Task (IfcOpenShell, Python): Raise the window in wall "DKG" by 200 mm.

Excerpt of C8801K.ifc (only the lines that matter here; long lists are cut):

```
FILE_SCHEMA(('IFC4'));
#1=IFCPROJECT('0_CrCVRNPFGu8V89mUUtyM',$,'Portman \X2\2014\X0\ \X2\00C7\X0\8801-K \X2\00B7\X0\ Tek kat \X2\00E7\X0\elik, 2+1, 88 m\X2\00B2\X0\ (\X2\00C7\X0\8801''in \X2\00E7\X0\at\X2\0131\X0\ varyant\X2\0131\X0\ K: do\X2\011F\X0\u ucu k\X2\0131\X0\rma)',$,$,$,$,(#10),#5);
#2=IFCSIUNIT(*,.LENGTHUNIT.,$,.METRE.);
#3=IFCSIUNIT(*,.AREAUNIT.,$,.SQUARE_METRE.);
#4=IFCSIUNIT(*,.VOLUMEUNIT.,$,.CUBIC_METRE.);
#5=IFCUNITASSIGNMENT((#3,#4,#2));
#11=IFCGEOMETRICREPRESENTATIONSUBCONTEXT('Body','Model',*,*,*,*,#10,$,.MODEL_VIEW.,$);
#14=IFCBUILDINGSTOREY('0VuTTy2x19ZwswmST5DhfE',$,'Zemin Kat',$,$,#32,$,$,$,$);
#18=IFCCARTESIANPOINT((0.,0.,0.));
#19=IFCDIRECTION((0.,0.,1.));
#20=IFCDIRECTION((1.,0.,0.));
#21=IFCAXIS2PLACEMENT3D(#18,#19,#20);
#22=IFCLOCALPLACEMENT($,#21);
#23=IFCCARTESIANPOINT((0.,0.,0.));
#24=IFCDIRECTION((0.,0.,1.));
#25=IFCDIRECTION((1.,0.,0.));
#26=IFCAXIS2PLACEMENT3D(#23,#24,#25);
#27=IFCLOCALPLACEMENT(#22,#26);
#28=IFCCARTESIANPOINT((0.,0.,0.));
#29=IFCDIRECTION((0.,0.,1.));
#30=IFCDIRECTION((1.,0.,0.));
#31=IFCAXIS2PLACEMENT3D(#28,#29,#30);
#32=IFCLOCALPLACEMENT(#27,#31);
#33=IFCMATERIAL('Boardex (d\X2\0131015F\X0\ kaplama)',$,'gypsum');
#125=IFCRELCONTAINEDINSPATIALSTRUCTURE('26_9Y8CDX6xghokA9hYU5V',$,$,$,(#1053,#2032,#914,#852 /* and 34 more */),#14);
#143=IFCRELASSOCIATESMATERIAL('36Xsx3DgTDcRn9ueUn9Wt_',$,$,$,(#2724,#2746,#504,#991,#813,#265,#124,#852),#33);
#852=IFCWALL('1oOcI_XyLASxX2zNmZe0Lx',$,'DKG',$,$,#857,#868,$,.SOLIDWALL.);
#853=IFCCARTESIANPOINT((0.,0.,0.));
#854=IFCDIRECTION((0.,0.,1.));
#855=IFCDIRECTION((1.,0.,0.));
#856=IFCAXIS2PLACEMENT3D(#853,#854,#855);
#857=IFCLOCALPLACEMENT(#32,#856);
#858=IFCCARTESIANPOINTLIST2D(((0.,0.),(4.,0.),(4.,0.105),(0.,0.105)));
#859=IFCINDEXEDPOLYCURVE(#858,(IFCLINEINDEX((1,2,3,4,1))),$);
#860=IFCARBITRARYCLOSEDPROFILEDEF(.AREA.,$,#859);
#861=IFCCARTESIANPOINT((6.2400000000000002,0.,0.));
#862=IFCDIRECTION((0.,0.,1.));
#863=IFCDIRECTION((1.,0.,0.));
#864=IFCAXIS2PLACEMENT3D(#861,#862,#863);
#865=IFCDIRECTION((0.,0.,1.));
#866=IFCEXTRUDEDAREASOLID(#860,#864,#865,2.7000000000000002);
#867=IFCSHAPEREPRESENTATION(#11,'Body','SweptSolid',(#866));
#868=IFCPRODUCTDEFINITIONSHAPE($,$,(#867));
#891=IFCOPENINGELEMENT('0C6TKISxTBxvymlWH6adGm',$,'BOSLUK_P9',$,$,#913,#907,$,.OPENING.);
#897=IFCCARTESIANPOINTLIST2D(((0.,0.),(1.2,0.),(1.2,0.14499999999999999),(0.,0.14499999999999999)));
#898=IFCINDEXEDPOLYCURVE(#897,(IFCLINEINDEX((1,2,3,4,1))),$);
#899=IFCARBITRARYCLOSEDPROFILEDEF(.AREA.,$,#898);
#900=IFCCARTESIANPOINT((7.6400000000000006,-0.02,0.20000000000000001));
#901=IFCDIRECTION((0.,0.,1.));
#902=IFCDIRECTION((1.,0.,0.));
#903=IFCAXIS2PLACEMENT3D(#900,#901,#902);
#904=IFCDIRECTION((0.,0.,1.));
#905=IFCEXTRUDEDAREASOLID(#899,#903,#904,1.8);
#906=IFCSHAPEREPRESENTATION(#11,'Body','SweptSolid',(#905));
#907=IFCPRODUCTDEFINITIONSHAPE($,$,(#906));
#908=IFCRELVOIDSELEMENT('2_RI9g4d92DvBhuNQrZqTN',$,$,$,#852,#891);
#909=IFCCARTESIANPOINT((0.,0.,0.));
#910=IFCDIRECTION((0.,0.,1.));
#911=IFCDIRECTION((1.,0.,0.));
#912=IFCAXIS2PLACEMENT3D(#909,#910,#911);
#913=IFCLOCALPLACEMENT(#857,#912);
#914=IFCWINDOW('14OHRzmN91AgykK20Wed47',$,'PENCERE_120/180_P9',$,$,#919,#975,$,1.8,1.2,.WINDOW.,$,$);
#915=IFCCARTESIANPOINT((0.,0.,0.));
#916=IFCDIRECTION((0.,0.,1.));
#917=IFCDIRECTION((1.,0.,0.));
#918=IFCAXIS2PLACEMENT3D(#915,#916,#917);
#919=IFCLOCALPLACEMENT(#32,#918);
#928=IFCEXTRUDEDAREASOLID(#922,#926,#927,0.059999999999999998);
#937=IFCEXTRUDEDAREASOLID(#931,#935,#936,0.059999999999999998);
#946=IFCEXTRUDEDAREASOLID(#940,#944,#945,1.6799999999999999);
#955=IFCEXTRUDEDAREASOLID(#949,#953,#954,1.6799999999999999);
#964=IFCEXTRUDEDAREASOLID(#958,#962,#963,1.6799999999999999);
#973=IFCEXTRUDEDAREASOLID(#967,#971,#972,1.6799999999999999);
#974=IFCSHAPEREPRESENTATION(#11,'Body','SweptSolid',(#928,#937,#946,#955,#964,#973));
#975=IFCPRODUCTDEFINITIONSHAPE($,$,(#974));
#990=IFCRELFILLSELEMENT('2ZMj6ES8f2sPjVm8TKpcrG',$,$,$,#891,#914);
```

```python
import numpy as np
import ifcopenshell
import ifcopenshell.api.geometry
import ifcopenshell.util.placement
import ifcopenshell.util.unit

model = ifcopenshell.open("C8801K.ifc")
unit_scale = ifcopenshell.util.unit.calculate_unit_scale(model)

window = model.by_guid("14OHRzmN91AgykK20Wed47")
opening = window.FillsVoids[0].RelatingOpeningElement
dz = 0.2 / unit_scale

shift = np.array([0.0, 0.0, dz])
# The window is not placed relative to its opening, so move both.
for product in (opening, window):
    matrix = ifcopenshell.util.placement.get_local_placement(product.ObjectPlacement)
    matrix[:3, 3] += shift
    ifcopenshell.api.geometry.edit_object_placement(model, product=product, matrix=matrix, is_si=False)

print(f"moved by {dz * unit_scale:+.3f} m")

model.write("C8801K_updated.ifc")
```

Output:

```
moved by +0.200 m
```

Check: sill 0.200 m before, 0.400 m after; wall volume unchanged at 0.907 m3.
